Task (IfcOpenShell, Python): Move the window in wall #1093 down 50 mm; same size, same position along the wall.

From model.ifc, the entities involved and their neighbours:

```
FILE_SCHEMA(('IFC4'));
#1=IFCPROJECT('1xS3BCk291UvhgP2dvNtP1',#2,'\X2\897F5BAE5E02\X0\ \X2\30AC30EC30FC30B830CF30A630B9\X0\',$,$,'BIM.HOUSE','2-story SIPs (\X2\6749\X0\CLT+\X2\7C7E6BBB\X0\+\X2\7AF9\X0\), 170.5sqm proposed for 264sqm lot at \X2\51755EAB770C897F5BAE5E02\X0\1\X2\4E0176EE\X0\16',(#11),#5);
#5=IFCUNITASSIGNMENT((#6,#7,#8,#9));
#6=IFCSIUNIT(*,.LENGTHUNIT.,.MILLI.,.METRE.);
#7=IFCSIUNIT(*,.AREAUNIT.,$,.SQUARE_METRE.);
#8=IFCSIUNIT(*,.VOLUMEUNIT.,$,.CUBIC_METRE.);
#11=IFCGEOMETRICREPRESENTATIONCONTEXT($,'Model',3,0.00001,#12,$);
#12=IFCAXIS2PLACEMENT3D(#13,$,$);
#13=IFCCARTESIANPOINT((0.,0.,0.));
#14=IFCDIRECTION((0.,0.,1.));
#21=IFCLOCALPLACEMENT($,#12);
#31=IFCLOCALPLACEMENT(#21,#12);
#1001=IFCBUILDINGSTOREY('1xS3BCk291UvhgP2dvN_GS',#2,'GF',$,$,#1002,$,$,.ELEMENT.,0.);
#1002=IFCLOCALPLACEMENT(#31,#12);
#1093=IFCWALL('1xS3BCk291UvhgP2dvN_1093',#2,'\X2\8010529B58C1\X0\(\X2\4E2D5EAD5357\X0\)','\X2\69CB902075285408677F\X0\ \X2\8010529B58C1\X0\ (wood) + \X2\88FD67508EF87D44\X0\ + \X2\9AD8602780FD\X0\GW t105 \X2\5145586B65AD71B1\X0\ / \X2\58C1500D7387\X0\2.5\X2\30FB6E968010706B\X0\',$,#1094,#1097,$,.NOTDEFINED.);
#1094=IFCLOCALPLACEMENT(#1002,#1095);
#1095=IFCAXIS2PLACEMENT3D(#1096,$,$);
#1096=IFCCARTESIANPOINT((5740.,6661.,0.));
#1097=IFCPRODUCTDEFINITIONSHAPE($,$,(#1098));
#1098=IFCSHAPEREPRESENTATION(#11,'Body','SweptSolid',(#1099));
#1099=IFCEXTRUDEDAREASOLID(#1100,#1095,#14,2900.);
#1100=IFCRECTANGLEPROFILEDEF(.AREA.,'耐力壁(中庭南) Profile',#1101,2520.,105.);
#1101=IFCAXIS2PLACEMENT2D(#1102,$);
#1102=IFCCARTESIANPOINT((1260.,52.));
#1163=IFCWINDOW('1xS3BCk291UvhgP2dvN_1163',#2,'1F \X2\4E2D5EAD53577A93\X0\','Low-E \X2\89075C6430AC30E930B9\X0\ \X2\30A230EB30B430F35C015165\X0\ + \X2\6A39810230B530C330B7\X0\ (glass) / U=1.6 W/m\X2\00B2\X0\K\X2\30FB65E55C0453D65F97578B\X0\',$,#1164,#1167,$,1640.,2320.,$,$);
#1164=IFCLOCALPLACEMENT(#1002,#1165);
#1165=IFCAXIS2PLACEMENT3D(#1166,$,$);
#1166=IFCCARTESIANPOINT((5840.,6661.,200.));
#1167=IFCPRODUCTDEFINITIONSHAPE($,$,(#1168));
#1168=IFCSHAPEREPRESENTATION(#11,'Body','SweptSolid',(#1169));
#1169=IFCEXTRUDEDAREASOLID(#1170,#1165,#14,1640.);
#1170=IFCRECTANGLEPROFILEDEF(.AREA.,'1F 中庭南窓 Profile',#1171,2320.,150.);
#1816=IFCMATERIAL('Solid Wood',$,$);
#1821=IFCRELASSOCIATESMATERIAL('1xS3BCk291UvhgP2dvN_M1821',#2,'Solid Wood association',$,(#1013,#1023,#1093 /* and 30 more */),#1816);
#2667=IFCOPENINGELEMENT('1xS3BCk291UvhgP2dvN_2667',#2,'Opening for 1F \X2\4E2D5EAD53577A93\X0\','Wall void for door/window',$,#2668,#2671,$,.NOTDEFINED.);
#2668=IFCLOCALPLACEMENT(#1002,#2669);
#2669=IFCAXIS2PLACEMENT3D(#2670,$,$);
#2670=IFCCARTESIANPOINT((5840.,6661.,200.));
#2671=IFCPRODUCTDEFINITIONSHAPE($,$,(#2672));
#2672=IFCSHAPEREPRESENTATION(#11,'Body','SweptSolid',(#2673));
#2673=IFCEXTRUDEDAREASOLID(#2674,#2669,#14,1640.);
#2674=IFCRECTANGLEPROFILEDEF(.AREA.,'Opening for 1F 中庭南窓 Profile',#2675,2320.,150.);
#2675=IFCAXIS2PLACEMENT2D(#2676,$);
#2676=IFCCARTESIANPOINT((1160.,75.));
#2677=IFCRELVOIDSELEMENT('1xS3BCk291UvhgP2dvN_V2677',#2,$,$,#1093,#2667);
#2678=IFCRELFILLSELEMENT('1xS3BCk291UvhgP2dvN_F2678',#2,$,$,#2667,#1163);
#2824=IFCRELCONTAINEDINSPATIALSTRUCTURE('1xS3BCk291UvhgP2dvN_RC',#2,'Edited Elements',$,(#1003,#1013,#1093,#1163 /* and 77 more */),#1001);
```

```python
import numpy as np
import ifcopenshell
import ifcopenshell.api.geometry
import ifcopenshell.util.placement
import ifcopenshell.util.unit

model = ifcopenshell.open("model.ifc")
unit_scale = ifcopenshell.util.unit.calculate_unit_scale(model)

window = model.by_guid("1xS3BCk291UvhgP2dvN_1163")
opening = window.FillsVoids[0].RelatingOpeningElement
dz = -0.05 / unit_scale

shift = np.array([0.0, 0.0, dz])
# The window is not placed relative to its opening, so move both.
for product in (opening, window):
    matrix = ifcopenshell.util.placement.get_local_placement(product.ObjectPlacement)
    matrix[:3, 3] += shift
    ifcopenshell.api.geometry.edit_object_placement(model, product=product, matrix=matrix, is_si=False)

print(f"moved by {dz * unit_scale:+.3f} m")

model.write("model_v2.ifc")
```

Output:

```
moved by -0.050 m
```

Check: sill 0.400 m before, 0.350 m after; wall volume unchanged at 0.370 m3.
